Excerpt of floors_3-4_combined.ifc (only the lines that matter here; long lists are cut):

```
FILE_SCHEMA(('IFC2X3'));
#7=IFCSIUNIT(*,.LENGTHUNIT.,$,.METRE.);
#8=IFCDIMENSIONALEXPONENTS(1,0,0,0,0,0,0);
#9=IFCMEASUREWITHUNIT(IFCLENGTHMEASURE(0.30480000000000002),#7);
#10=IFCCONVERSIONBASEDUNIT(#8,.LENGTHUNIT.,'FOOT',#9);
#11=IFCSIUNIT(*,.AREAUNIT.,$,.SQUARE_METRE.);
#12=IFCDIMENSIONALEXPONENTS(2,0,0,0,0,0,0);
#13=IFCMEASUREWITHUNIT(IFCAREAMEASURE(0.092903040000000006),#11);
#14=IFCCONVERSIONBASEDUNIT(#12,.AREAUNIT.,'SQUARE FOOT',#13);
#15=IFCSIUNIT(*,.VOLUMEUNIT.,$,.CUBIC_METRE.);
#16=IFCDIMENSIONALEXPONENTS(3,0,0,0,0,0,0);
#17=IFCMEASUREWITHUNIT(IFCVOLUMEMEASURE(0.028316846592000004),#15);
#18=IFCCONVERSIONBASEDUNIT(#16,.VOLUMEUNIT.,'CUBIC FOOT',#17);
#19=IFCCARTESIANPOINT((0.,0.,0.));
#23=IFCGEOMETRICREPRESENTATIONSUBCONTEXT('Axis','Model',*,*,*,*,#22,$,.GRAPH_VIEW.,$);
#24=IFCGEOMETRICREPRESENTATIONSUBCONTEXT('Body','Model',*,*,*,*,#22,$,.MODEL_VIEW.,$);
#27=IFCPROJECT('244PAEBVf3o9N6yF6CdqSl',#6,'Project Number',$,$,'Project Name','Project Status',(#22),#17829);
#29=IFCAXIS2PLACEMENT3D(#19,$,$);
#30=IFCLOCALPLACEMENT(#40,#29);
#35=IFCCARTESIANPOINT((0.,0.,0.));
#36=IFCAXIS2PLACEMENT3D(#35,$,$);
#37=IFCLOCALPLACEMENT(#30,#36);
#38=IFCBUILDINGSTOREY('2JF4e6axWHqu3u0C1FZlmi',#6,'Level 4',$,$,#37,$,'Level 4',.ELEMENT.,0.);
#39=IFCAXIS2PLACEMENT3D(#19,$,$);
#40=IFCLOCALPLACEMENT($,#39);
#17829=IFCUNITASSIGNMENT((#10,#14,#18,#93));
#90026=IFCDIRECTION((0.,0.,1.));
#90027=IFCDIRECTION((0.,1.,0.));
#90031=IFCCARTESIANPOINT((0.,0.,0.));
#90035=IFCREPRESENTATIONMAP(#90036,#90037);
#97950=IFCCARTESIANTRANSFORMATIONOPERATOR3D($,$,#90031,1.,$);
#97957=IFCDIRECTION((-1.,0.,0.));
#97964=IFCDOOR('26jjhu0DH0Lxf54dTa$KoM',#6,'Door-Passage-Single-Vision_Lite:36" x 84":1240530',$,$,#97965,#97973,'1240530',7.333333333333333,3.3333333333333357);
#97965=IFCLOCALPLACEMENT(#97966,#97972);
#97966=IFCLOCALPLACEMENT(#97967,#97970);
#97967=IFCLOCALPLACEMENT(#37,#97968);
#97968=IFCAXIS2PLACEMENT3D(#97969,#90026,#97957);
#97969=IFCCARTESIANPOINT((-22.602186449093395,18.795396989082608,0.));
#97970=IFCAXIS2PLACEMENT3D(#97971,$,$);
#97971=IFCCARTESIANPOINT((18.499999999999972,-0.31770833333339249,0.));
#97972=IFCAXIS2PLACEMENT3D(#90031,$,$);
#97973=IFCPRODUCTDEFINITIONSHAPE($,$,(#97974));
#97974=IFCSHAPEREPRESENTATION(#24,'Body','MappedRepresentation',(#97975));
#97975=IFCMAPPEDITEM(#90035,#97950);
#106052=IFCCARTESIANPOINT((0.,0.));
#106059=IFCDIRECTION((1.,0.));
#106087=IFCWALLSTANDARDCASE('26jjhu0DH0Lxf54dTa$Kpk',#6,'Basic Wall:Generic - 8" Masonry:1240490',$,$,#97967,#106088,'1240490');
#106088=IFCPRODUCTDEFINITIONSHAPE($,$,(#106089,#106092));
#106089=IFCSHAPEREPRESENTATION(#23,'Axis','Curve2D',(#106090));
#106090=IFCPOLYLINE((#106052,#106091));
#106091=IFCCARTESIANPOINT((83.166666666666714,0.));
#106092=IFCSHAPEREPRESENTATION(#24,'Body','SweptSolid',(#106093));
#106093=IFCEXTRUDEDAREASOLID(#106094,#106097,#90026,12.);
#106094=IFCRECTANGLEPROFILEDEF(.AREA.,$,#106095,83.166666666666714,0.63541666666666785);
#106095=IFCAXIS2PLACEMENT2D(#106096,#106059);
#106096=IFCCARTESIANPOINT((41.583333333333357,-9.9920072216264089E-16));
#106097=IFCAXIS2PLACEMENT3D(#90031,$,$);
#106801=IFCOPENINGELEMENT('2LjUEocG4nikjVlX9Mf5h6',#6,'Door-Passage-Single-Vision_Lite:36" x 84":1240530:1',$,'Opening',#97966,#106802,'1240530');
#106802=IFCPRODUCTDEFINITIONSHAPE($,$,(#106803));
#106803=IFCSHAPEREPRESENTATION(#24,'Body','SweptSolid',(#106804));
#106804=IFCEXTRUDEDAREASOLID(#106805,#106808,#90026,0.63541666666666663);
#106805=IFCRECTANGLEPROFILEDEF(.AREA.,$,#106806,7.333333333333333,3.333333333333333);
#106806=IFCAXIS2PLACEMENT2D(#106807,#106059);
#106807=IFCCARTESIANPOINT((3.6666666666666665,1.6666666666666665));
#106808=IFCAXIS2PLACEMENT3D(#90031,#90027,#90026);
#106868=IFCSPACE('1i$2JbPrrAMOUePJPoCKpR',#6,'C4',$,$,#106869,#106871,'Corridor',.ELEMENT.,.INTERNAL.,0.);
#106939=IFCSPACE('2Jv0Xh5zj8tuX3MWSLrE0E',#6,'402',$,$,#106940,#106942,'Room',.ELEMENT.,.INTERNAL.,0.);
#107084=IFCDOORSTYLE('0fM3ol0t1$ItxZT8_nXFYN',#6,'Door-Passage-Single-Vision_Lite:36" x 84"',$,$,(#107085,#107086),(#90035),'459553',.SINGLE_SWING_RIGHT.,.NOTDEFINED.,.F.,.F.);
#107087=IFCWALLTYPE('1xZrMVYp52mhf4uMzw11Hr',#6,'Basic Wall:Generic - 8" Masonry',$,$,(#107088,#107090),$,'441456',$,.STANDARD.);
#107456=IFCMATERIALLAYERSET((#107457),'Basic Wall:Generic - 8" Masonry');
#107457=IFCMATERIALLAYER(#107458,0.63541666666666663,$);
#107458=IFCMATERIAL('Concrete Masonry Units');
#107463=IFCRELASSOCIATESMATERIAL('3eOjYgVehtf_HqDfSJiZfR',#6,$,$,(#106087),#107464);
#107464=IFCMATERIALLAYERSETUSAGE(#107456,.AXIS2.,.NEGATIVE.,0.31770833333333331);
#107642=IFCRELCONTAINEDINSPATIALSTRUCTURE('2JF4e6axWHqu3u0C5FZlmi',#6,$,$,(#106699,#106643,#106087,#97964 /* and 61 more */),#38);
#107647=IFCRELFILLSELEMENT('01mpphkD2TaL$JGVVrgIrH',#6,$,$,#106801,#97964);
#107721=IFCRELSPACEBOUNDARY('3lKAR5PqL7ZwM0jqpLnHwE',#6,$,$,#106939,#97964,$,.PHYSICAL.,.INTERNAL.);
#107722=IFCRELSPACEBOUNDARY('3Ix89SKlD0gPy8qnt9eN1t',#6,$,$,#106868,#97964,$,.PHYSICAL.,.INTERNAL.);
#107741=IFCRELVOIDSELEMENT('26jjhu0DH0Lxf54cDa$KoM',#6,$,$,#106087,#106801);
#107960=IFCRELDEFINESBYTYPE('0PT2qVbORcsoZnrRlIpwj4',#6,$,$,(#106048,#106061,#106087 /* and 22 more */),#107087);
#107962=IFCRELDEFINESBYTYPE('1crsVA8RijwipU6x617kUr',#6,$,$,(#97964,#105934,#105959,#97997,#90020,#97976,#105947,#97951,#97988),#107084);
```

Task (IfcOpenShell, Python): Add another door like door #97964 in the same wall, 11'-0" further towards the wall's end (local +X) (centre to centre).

```python
import ifcopenshell
import ifcopenshell.api.feature
import ifcopenshell.api.geometry
import ifcopenshell.api.root
import ifcopenshell.geom
import ifcopenshell.util.element
import ifcopenshell.util.placement
import ifcopenshell.util.shape
import ifcopenshell.util.unit

model = ifcopenshell.open("floors_3-4_combined.ifc")
unit_scale = ifcopenshell.util.unit.calculate_unit_scale(model)
settings = ifcopenshell.geom.settings()


def volume(element):
    """Net volume in cubic metres, openings subtracted."""
    shape = ifcopenshell.geom.create_shape(settings, element)
    return ifcopenshell.util.shape.get_volume(shape.geometry)


def reuse_history(source, copy):
    """copy_class also copies each property set's owner history, people and application; keep the originals."""
    for rel in copy.IsDefinedBy:
        if rel.is_a("IfcRelDefinesByProperties") and (history := rel.RelatingPropertyDefinition.OwnerHistory):
            rel.RelatingPropertyDefinition.OwnerHistory = source.OwnerHistory
            ifcopenshell.util.element.remove_deep2(model, history)


door = model.by_id(97964)
opening = door.FillsVoids[0].RelatingOpeningElement
wall = opening.VoidsElements[0].RelatingBuildingElement
before = volume(wall)
shift = ifcopenshell.util.placement.get_local_placement(wall.ObjectPlacement)[:3, 0] * 132 * 0.0254 / unit_scale

# copy_class copies the void relationship, type, container and properties, but no geometry.
new_opening = ifcopenshell.api.root.copy_class(model, product=opening)
new_opening.Representation = ifcopenshell.util.element.copy_deep(
    model, opening.Representation, exclude=["IfcGeometricRepresentationContext", "IfcRepresentationMap"]
)
new_opening.Name = 'Door-Passage-Single-Vision_Lite:36" x 84"'
new_opening.Tag = None
new_door = ifcopenshell.api.root.copy_class(model, product=door)
new_door.Representation = ifcopenshell.util.element.copy_deep(
    model, door.Representation, exclude=["IfcGeometricRepresentationContext", "IfcRepresentationMap"]
)
new_door.Name = 'Door-Passage-Single-Vision_Lite:36" x 84"'
new_door.Tag = None
reuse_history(door, new_door)
fills = ifcopenshell.api.feature.add_filling(model, opening=new_opening, element=new_door)
fills.OwnerHistory = new_door.OwnerHistory  # required in IFC2X3

for old, new in ((opening, new_opening), (door, new_door)):
    matrix = ifcopenshell.util.placement.get_local_placement(old.ObjectPlacement)
    matrix[:3, 3] += shift
    ifcopenshell.api.geometry.edit_object_placement(model, product=new, matrix=matrix, is_si=False)

after = volume(wall)

print(f"wall volume {before:.3f} -> {after:.3f} m3")

model.write("floors_3-4_combined_updated.ifc")
```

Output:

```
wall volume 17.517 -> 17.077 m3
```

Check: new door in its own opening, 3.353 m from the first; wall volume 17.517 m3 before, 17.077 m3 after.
